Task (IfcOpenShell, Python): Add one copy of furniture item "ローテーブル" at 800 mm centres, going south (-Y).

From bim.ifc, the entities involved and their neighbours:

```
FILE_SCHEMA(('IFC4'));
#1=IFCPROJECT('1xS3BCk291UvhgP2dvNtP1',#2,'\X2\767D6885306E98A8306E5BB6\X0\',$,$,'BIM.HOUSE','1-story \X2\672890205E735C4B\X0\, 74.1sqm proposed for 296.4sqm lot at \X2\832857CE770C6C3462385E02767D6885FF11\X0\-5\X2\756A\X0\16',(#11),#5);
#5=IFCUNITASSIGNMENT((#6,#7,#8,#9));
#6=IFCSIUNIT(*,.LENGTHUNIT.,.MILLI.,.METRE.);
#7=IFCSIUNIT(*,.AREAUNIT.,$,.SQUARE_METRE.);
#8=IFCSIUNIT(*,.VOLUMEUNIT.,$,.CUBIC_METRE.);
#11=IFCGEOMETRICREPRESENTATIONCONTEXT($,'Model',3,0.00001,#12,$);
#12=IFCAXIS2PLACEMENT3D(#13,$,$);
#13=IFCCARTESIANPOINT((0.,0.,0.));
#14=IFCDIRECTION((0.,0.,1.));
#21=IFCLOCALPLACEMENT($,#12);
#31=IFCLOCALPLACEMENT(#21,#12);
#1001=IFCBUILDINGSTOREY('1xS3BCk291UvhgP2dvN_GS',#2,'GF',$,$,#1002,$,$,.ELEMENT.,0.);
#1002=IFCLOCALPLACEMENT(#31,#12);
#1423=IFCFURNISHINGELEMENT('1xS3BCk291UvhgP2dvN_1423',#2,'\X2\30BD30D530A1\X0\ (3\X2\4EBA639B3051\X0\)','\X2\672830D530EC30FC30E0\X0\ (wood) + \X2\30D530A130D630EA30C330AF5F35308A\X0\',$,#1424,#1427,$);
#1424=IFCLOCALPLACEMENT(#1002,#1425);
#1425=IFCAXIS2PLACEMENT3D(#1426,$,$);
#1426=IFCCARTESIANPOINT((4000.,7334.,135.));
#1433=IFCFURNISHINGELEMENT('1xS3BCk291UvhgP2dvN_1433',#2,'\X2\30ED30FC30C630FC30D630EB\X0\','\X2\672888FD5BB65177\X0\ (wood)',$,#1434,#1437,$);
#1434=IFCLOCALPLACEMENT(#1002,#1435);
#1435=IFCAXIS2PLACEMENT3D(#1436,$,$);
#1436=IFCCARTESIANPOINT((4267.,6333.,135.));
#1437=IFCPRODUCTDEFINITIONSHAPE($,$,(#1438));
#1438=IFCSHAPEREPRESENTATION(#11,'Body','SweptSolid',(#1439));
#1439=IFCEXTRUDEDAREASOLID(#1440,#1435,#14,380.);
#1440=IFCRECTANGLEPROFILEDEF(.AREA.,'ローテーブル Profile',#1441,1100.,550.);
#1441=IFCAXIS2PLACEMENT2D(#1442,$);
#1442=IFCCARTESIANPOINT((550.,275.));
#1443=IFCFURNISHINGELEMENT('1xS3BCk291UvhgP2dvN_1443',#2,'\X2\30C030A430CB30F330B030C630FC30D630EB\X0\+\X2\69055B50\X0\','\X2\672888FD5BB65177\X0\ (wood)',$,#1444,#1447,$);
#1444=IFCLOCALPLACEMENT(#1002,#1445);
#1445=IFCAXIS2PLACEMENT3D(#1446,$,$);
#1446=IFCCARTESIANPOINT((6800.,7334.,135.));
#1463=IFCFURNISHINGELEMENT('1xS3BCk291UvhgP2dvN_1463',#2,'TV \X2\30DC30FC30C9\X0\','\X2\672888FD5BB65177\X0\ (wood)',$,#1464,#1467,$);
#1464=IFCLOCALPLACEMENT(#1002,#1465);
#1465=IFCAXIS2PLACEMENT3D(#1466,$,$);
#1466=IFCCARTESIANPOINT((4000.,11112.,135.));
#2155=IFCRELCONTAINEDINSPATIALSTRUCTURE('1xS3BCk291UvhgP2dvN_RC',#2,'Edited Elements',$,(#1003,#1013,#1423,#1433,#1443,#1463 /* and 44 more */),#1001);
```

```python
import numpy as np
import ifcopenshell
import ifcopenshell.api.geometry
import ifcopenshell.api.root
import ifcopenshell.util.element
import ifcopenshell.util.placement
import ifcopenshell.util.unit

model = ifcopenshell.open("bim.ifc")
unit_scale = ifcopenshell.util.unit.calculate_unit_scale(model)


def reuse_history(source, copy):
    """copy_class also copies each property set's owner history, people and application; keep the originals."""
    for rel in copy.IsDefinedBy:
        if rel.is_a("IfcRelDefinesByProperties") and (history := rel.RelatingPropertyDefinition.OwnerHistory):
            rel.RelatingPropertyDefinition.OwnerHistory = source.OwnerHistory
            ifcopenshell.util.element.remove_deep2(model, history)


source = model.by_guid("1xS3BCk291UvhgP2dvN_1433")
base = ifcopenshell.util.placement.get_local_placement(source.ObjectPlacement)
step = np.array([0.0, -1.0, 0.0]) * 0.8 / unit_scale

for i in range(1, 2):
    copy = ifcopenshell.api.root.copy_class(model, product=source)
    copy.Representation = ifcopenshell.util.element.copy_deep(
        model, source.Representation, exclude=["IfcGeometricRepresentationContext", "IfcRepresentationMap"]
    )
    reuse_history(source, copy)
    matrix = base.copy()
    matrix[:3, 3] += i * step
    print("added at", matrix[:3, 3].round(3) + 0.0)
    ifcopenshell.api.geometry.edit_object_placement(model, product=copy, matrix=matrix, is_si=False)

model.write("bim_edited.ifc")
```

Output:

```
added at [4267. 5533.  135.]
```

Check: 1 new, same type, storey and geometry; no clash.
